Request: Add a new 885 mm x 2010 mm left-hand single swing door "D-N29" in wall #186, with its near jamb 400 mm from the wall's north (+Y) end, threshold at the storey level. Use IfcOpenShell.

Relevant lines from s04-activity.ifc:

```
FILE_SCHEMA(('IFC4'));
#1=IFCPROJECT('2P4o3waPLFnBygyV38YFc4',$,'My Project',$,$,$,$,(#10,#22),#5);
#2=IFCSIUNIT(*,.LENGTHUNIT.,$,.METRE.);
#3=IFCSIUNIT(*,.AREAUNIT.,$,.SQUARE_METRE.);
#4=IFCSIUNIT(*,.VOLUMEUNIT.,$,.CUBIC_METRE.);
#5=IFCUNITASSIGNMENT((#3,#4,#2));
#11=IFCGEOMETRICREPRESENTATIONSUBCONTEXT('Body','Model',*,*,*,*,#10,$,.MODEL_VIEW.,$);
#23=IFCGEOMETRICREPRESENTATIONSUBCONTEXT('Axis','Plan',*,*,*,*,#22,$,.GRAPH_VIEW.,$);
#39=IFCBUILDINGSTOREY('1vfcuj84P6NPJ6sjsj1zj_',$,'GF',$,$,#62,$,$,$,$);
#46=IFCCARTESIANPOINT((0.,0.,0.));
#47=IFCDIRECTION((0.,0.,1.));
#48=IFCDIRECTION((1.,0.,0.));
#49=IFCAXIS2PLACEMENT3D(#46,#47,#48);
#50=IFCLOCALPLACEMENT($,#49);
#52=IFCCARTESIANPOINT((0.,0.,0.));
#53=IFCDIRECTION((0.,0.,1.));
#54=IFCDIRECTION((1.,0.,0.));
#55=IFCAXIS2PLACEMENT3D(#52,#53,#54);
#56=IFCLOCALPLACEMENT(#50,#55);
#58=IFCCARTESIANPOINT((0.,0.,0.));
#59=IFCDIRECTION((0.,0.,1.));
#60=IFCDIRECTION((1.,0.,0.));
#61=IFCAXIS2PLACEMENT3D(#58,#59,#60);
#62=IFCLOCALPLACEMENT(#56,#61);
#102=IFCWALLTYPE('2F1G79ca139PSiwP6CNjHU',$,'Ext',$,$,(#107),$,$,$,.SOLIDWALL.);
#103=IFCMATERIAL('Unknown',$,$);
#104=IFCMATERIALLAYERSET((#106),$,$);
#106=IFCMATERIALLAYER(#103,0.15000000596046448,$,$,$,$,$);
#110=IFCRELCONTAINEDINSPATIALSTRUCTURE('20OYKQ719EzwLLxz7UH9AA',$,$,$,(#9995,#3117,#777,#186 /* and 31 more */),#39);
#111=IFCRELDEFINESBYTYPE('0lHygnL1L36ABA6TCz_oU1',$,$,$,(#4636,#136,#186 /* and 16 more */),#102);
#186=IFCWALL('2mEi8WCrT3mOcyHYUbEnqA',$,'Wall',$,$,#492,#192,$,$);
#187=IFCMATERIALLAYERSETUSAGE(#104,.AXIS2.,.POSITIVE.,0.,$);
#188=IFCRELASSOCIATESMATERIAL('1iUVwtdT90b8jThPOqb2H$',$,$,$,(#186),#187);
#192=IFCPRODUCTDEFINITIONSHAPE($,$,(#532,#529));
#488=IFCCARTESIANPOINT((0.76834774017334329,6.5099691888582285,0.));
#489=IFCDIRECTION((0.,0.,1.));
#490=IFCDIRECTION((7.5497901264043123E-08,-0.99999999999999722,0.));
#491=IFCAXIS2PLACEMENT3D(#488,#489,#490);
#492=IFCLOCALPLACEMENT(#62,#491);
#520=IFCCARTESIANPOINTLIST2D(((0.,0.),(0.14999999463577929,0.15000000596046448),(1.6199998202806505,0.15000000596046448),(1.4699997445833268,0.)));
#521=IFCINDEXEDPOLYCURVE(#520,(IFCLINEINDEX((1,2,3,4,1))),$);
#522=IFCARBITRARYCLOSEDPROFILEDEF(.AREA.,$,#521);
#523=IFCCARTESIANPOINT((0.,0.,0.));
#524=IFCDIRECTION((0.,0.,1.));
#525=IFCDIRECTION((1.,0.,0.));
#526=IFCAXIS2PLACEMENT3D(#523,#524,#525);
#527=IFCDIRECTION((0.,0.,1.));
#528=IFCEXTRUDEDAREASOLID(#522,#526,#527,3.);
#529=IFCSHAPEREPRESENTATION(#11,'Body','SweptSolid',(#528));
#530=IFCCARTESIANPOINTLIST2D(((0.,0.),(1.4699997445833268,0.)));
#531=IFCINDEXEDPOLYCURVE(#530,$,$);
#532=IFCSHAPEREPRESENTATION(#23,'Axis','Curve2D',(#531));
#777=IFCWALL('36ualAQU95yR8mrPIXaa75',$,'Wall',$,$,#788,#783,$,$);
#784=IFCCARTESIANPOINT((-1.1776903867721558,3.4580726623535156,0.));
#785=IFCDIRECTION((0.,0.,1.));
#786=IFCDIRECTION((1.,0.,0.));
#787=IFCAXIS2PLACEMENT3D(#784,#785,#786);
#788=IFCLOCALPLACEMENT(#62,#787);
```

```python
import numpy as np
import ifcopenshell
import ifcopenshell.api.feature
import ifcopenshell.api.geometry
import ifcopenshell.api.root
import ifcopenshell.api.spatial
import ifcopenshell.geom
import ifcopenshell.util.element
import ifcopenshell.util.placement
import ifcopenshell.util.representation
import ifcopenshell.util.shape
import ifcopenshell.util.unit

model = ifcopenshell.open("s04-activity.ifc")
unit_scale = ifcopenshell.util.unit.calculate_unit_scale(model)
settings = ifcopenshell.geom.settings()


def volume(element):
    """Net volume in cubic metres, openings subtracted."""
    shape = ifcopenshell.geom.create_shape(settings, element)
    return ifcopenshell.util.shape.get_volume(shape.geometry)


wall = model.by_guid("2mEi8WCrT3mOcyHYUbEnqA")
storey = ifcopenshell.util.element.get_container(wall, ifc_class="IfcBuildingStorey")
context = ifcopenshell.util.representation.get_context(model, "Model", "Body", "MODEL_VIEW")
before = volume(wall)

width, height, from_end, sill = 0.885, 2.01, 0.4, 0.0  # metres

# The wall runs along its own X axis, and the end named is its -X end.
wall_shape = ifcopenshell.geom.create_shape(settings, wall)
x, y, z = ifcopenshell.util.shape.get_vertices(wall_shape.geometry).T
start = x.min() + from_end
face, thickness = float(y.min()), float(y.max() - y.min())
wall_matrix = ifcopenshell.util.placement.get_local_placement(wall.ObjectPlacement)
level = ifcopenshell.util.placement.get_local_placement(storey.ObjectPlacement)[2, 3]


def in_wall(x, y):
    """Placement at x, y metres in the wall's axes, at sill height."""
    matrix = wall_matrix.copy()
    matrix[:, 3] = wall_matrix @ np.array([x / unit_scale, y / unit_scale, 0.0, 1.0])
    matrix[2, 3] = level + sill / unit_scale
    return matrix


# Opening: a box that overshoots both wall faces by 50 mm.
opening = ifcopenshell.api.root.create_entity(model, ifc_class="IfcOpeningElement", predefined_type="OPENING")
box = ifcopenshell.api.geometry.add_wall_representation(
    model, context=context, length=width, height=height, thickness=thickness + 0.1
)
ifcopenshell.api.geometry.assign_representation(model, product=opening, representation=box)
ifcopenshell.api.geometry.edit_object_placement(model, product=opening, matrix=in_wall(start, face - 0.05), is_si=False)
ifcopenshell.api.feature.add_feature(model, feature=opening, element=wall)

door = ifcopenshell.api.root.create_entity(model, ifc_class="IfcDoor", name="D-N29", predefined_type="DOOR")
door.OverallWidth, door.OverallHeight = width / unit_scale, height / unit_scale
door.OperationType = "SINGLE_SWING_LEFT"
body = ifcopenshell.api.geometry.add_door_representation(
    model,
    context=context,
    overall_width=door.OverallWidth,
    overall_height=door.OverallHeight,
    operation_type="SINGLE_SWING_LEFT",
    lining_properties={"LiningDepth": thickness / unit_scale, "ThresholdDepth": thickness / unit_scale},
)
ifcopenshell.api.geometry.assign_representation(model, product=door, representation=body)
ifcopenshell.api.spatial.assign_container(model, products=[door], relating_structure=storey)
ifcopenshell.api.feature.add_filling(model, opening=opening, element=door)

# The lining spans the wall, so the door starts at the wall face.
ifcopenshell.api.geometry.edit_object_placement(model, product=door, matrix=in_wall(start, face), is_si=False)

after = volume(wall)

print(f"wall volume {before:.3f} -> {after:.3f} m3")

model.write("s04-activity_edited.ifc")
```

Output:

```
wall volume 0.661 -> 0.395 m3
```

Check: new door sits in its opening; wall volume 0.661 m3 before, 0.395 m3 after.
